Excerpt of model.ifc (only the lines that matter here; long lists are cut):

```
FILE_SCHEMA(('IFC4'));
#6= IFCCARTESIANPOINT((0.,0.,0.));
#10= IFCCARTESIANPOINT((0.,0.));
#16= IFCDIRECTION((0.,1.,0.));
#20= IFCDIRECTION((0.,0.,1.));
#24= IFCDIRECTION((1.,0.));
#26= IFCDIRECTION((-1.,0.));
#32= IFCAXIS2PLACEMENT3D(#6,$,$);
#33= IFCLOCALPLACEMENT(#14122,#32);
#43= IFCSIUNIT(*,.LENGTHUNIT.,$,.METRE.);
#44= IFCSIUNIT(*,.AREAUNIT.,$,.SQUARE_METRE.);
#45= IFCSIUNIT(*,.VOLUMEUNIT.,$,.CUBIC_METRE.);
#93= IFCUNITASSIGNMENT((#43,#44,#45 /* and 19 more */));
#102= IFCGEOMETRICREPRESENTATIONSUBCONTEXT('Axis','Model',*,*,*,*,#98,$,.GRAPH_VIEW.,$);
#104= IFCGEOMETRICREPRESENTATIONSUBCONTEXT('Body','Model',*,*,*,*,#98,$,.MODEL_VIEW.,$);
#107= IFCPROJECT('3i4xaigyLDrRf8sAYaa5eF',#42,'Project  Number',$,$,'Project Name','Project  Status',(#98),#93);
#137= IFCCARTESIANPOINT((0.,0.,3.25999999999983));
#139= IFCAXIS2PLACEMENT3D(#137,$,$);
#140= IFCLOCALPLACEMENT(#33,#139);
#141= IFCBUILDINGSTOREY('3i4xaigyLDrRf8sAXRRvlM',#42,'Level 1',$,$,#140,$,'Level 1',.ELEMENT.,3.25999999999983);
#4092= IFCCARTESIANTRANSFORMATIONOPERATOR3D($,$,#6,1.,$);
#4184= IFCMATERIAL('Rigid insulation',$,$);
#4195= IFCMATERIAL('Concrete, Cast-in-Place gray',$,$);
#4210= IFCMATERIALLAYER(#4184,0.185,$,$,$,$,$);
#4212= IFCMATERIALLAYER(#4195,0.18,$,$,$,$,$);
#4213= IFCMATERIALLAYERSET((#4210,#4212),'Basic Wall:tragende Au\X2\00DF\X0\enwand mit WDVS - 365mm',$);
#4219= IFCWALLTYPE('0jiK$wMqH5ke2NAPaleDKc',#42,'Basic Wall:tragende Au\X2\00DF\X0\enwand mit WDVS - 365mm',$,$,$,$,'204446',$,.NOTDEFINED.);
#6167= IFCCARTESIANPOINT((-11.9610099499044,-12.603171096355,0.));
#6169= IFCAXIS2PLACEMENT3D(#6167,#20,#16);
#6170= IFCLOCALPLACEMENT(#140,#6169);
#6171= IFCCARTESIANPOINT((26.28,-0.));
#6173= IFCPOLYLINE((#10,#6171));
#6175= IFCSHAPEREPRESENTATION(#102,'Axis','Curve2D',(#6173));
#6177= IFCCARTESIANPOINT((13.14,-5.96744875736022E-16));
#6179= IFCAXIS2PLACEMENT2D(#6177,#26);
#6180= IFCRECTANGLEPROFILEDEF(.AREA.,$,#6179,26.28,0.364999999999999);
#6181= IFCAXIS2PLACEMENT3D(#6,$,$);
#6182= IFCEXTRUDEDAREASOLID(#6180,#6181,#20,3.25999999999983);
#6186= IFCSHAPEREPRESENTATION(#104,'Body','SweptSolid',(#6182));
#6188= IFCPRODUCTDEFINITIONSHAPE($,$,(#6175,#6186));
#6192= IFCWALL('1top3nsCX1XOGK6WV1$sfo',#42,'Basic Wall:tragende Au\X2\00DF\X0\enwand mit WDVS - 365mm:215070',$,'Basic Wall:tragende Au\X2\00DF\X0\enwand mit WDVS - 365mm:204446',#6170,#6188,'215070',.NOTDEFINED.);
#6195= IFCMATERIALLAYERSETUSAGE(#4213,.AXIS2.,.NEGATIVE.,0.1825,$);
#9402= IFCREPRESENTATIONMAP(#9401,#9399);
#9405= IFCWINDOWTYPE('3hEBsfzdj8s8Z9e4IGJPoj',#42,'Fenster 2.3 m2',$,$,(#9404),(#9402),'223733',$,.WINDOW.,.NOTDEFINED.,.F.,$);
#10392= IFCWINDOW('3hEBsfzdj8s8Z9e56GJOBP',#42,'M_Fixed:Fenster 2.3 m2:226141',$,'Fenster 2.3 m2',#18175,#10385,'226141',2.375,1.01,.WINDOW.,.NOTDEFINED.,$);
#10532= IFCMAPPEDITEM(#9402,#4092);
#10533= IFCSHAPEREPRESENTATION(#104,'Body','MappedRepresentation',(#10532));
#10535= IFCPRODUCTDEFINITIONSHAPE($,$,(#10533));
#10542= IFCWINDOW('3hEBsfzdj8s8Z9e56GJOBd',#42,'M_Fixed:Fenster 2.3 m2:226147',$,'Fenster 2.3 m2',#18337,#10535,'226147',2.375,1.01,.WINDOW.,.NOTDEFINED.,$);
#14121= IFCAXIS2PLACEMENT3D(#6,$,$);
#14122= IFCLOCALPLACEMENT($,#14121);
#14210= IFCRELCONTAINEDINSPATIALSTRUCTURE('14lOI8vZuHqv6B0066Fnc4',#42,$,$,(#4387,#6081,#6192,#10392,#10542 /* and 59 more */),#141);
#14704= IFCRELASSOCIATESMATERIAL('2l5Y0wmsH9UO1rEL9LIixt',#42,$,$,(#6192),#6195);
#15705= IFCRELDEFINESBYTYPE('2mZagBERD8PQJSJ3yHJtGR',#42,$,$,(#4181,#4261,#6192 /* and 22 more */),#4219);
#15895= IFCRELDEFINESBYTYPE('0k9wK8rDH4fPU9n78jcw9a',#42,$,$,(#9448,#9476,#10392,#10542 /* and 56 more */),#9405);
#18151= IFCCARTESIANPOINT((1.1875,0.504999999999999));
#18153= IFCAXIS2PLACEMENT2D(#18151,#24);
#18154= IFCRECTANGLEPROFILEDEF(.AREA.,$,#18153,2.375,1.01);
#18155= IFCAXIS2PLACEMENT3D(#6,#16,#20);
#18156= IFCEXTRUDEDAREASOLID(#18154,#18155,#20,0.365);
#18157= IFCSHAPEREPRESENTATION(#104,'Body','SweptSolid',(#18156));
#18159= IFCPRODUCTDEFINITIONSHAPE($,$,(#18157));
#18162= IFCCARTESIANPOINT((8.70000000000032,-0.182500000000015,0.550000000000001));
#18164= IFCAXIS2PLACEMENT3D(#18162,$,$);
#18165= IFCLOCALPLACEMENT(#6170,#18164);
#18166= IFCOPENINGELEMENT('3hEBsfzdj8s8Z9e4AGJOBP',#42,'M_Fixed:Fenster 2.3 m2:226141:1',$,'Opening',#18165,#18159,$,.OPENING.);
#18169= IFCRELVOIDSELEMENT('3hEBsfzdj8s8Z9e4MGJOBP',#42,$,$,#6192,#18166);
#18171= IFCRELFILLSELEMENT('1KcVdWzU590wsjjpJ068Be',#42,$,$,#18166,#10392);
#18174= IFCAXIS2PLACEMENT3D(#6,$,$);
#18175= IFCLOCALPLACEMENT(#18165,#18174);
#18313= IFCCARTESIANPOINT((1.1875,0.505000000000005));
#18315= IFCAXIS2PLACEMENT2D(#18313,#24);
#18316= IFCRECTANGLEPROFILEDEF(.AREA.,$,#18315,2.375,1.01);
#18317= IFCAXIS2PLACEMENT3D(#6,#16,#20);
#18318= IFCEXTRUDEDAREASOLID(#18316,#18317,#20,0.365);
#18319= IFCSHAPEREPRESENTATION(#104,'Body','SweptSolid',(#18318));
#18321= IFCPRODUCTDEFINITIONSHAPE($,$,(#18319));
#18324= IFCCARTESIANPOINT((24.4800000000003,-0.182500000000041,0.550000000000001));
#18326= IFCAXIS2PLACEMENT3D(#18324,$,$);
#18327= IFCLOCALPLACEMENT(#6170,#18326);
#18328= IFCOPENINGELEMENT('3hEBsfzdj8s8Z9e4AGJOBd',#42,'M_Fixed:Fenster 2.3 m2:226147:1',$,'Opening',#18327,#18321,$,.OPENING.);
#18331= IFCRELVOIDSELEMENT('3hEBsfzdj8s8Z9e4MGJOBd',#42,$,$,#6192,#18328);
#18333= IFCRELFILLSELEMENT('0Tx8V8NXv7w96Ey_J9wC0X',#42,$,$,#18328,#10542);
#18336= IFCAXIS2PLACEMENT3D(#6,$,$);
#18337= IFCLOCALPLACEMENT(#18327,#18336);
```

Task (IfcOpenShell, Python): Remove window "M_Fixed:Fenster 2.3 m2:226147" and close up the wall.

```python
import ifcopenshell
import ifcopenshell.api.feature
import ifcopenshell.api.root
import ifcopenshell.geom
import ifcopenshell.util.shape

model = ifcopenshell.open("model.ifc")
settings = ifcopenshell.geom.settings()


def volume(element):
    """Net volume in cubic metres, openings subtracted."""
    shape = ifcopenshell.geom.create_shape(settings, element)
    return ifcopenshell.util.shape.get_volume(shape.geometry)


window = model.by_id(10542)
opening = window.FillsVoids[0].RelatingOpeningElement
wall = opening.VoidsElements[0].RelatingBuildingElement
before = volume(wall)

ifcopenshell.api.root.remove_product(model, product=window)
ifcopenshell.api.feature.remove_feature(model, feature=opening)

after = volume(wall)

print(f"wall volume {before:.3f} -> {after:.3f} m3")

model.write("model_edited.ifc")
```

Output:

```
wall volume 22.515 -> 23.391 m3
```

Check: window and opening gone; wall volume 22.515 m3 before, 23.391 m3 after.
